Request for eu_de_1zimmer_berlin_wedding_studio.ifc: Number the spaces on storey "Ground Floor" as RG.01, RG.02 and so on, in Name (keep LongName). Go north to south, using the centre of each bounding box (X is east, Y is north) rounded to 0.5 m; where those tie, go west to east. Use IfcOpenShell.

First a look at what the model holds.

```python
import ifcopenshell
import ifcopenshell.util.element
import ifcopenshell.util.placement

model = ifcopenshell.open("eu_de_1zimmer_berlin_wedding_studio.ifc")
print(model.schema)
storey = next(s for s in model.by_type("IfcBuildingStorey") if s.Name == "Ground Floor")
spaces = [e for e in ifcopenshell.util.element.get_decomposition(storey) if e.is_a("IfcSpace")]
for e in sorted(spaces, key=lambda e: e.id()):
    origin = ifcopenshell.util.placement.get_local_placement(e.ObjectPlacement)[:3, 3]
    print(e.id(), e.Name, e.LongName, origin.round(2) + 0.0, sep=" | ")
```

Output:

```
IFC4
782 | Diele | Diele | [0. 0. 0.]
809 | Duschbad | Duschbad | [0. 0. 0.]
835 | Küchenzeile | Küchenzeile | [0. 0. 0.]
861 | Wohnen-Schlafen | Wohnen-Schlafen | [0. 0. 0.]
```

```python
import ifcopenshell
import ifcopenshell.geom
import ifcopenshell.util.element
import ifcopenshell.util.shape

model = ifcopenshell.open("eu_de_1zimmer_berlin_wedding_studio.ifc")
settings = ifcopenshell.geom.settings()
settings.set("use-world-coords", True)


def centre(element):
    shape = ifcopenshell.geom.create_shape(settings, element)
    return ifcopenshell.util.shape.get_bbox_centroid(shape.geometry)


storey = next(s for s in model.by_type("IfcBuildingStorey") if s.Name == "Ground Floor")
spaces = [e for e in ifcopenshell.util.element.get_decomposition(storey) if e.is_a("IfcSpace")]

# Insertion points can sit at a corner or the storey origin, so sort by the geometry (in metres).
centres = {e: centre(e) for e in spaces}
spaces.sort(key=lambda e: (-round(centres[e][1] / 0.5), centres[e][0]))

for i, e in enumerate(spaces, start=1):
    number = f"RG.{i:02d}"
    e.Name = number
    print(e.id(), number)

model.write("eu_de_1zimmer_berlin_wedding_studio_edited.ifc")
```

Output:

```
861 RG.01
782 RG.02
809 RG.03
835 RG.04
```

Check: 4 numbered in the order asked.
